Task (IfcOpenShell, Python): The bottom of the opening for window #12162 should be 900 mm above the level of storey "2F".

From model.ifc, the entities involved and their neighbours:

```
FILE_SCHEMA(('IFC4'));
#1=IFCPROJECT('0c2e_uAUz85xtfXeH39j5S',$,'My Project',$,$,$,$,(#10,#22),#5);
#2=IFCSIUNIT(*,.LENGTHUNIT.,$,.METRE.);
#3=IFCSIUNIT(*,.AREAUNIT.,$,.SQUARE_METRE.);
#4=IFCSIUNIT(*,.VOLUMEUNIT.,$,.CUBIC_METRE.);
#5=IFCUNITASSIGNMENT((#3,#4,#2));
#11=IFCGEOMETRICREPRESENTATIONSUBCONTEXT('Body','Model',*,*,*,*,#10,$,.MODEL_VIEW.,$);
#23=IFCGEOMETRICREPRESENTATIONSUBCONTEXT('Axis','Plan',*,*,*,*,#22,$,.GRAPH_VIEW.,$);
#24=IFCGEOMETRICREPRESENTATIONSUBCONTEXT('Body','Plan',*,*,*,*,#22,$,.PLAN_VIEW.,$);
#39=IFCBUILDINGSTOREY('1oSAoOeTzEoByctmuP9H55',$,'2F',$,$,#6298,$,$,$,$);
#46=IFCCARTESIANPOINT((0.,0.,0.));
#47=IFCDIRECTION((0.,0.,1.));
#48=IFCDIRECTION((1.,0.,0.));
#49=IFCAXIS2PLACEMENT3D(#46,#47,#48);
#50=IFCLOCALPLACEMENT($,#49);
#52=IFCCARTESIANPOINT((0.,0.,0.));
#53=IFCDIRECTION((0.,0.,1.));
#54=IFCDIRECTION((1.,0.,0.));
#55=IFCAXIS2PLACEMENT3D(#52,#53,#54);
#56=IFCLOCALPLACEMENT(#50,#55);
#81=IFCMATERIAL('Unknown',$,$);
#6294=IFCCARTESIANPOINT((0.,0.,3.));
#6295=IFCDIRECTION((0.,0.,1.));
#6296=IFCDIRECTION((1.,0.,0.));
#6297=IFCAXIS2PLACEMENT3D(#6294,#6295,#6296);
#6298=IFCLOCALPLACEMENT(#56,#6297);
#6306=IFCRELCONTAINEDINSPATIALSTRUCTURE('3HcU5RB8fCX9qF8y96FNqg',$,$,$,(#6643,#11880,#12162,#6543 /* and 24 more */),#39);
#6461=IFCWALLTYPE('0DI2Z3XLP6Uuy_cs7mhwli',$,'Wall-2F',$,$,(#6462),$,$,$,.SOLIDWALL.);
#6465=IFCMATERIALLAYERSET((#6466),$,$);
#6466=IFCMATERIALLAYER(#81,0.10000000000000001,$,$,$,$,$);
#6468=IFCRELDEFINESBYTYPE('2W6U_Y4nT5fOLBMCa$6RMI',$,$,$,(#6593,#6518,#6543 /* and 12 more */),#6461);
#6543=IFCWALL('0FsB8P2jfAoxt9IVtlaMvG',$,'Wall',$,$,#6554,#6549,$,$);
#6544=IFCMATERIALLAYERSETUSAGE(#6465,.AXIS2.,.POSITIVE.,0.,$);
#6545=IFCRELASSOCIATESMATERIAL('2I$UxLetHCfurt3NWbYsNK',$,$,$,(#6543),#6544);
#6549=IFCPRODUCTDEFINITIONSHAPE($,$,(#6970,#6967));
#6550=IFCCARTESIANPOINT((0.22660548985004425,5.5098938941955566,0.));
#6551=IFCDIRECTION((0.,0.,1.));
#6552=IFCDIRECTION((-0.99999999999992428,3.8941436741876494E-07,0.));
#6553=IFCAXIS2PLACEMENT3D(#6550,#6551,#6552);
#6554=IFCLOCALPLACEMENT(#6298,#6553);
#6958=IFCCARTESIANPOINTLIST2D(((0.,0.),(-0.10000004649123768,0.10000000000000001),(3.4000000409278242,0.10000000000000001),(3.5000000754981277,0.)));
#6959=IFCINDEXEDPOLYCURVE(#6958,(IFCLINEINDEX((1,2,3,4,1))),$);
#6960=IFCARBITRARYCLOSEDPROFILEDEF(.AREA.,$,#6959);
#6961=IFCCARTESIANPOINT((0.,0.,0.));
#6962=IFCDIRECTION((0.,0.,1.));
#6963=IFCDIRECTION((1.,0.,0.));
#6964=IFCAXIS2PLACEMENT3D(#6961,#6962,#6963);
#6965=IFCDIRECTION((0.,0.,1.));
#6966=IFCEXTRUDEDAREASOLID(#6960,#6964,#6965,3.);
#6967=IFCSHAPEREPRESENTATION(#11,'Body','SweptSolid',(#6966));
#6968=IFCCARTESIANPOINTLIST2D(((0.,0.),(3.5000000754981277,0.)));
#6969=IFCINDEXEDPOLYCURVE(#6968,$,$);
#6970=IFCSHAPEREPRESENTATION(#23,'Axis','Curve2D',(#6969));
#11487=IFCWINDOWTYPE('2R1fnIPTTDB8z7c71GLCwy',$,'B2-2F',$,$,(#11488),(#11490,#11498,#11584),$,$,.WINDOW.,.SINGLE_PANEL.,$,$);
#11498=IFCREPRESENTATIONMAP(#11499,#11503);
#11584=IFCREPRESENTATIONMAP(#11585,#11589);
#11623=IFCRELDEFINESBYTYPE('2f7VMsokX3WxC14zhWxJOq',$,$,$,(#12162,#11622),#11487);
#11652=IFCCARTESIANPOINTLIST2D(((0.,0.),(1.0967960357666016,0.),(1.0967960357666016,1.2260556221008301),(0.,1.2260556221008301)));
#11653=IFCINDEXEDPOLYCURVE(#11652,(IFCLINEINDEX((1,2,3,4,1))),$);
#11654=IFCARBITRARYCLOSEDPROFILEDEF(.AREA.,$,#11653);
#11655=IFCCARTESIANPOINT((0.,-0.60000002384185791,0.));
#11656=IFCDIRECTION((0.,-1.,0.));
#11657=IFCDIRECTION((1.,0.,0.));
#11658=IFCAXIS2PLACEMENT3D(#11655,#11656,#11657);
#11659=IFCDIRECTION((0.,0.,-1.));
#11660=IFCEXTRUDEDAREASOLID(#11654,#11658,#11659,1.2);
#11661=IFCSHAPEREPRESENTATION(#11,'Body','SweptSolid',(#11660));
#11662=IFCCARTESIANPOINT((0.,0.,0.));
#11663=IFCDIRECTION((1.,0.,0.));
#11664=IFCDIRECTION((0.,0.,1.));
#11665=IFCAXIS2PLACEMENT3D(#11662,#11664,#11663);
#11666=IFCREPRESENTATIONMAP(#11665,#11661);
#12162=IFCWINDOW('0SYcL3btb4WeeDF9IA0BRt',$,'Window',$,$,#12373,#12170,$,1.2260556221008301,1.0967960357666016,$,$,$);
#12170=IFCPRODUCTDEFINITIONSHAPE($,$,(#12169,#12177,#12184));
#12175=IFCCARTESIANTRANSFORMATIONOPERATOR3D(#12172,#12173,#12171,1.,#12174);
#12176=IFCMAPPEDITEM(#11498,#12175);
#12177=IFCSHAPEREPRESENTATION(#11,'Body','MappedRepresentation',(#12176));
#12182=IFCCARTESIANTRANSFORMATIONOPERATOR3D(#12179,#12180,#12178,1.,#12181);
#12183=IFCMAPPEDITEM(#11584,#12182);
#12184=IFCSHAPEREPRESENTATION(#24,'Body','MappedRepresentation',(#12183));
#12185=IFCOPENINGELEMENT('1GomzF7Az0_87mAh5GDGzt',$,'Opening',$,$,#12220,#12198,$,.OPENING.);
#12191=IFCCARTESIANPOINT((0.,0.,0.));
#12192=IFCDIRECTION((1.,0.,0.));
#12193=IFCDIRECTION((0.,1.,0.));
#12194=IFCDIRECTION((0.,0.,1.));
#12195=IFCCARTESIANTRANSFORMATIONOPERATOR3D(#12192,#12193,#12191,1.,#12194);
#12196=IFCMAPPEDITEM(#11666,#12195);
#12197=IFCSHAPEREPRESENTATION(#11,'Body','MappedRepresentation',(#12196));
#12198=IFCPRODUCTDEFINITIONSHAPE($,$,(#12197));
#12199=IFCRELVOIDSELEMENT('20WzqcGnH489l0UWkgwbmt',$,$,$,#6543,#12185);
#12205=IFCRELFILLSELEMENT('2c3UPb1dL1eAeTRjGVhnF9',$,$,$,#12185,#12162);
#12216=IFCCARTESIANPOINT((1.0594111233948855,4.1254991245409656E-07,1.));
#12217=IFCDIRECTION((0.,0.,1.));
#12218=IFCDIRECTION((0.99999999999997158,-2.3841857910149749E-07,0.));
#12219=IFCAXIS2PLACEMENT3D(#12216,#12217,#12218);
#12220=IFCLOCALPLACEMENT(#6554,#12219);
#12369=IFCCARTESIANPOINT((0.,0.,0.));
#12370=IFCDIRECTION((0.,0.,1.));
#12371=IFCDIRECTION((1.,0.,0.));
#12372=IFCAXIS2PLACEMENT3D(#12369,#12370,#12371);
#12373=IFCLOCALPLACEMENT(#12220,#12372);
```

```python
import numpy as np
import ifcopenshell
import ifcopenshell.api.geometry
import ifcopenshell.geom
import ifcopenshell.util.element
import ifcopenshell.util.placement
import ifcopenshell.util.shape
import ifcopenshell.util.unit

model = ifcopenshell.open("model.ifc")
unit_scale = ifcopenshell.util.unit.calculate_unit_scale(model)

window = model.by_guid("0SYcL3btb4WeeDF9IA0BRt")
opening = window.FillsVoids[0].RelatingOpeningElement
storey = ifcopenshell.util.element.get_container(window, ifc_class="IfcBuildingStorey")
level = ifcopenshell.util.placement.get_local_placement(storey.ObjectPlacement)[2, 3]

# The opening's origin need not be at the sill, so measure its lowest point.
shape = ifcopenshell.geom.create_shape(ifcopenshell.geom.settings(), opening)
bottom = ifcopenshell.util.shape.get_shape_bottom_elevation(shape, shape.geometry) / unit_scale
dz = level + 0.9 / unit_scale - bottom

shift = np.array([0.0, 0.0, dz])
# The window is placed relative to its opening, so it follows when the opening moves.
matrix = ifcopenshell.util.placement.get_local_placement(opening.ObjectPlacement)
matrix[:3, 3] += shift
ifcopenshell.api.geometry.edit_object_placement(
    model, product=opening, matrix=matrix, is_si=False, should_transform_children=True
)

print(f"moved by {dz * unit_scale:+.3f} m")

model.write("model_v2.ifc")
```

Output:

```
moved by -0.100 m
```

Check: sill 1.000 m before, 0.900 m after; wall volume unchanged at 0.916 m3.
